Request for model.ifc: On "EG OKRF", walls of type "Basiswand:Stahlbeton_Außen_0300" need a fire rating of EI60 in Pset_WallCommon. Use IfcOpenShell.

First a look at what the model holds.

```python
import ifcopenshell
import ifcopenshell.util.element

model = ifcopenshell.open("model.ifc")
print(model.schema)
storey = next(s for s in model.by_type("IfcBuildingStorey") if s.Name == "EG OKRF")
walls = [e for e in ifcopenshell.util.element.get_decomposition(storey) if e.is_a("IfcWall")]
seen = {}
for e in walls:
    element_type = ifcopenshell.util.element.get_type(e)
    key = (element_type.Name if element_type != e and element_type else None, ifcopenshell.util.element.get_pset(e, "Pset_WallCommon", "FireRating"))
    seen[key] = seen.get(key, 0) + 1
for (name, value), count in sorted(seen.items(), key=str):
    print(count, "x", name, "|", value)
```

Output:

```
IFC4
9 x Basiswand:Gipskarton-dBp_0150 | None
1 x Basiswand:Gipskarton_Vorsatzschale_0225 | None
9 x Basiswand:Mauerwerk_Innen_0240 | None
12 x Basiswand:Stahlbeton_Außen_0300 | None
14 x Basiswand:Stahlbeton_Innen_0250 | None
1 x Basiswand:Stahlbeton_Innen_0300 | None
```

```python
import ifcopenshell
import ifcopenshell.api.pset
import ifcopenshell.util.element

model = ifcopenshell.open("model.ifc")

storey = next(s for s in model.by_type("IfcBuildingStorey") if s.Name == "EG OKRF")
walls = [e for e in ifcopenshell.util.element.get_decomposition(storey) if e.is_a("IfcWall")]

count = 0
for e in walls:
    element_type = ifcopenshell.util.element.get_type(e)
    if element_type in (None, e) or element_type.Name != "Basiswand:Stahlbeton_Außen_0300":
        continue
    # add_pset returns the element's existing set when there is one.
    pset = ifcopenshell.api.pset.add_pset(model, product=e, name="Pset_WallCommon")
    ifcopenshell.api.pset.edit_pset(model, pset=pset, properties={"FireRating": "EI60"})
    count += 1

print(count, "walls updated")

model.write("model_updated.ifc")
```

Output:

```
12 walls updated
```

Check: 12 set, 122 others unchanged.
